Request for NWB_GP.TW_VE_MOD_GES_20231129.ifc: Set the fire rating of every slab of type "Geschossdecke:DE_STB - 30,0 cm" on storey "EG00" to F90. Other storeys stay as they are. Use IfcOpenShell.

First a look at what the model holds.

```python
import ifcopenshell
import ifcopenshell.util.element

model = ifcopenshell.open("NWB_GP.TW_VE_MOD_GES_20231129.ifc")
print(model.schema)
storey = next(s for s in model.by_type("IfcBuildingStorey") if s.Name == "EG00")
slabs = [e for e in ifcopenshell.util.element.get_decomposition(storey) if e.is_a("IfcSlab")]
seen = {}
for e in slabs:
    element_type = ifcopenshell.util.element.get_type(e)
    key = (element_type.Name if element_type != e and element_type else None, ifcopenshell.util.element.get_pset(e, "Pset_SlabCommon", "FireRating"))
    seen[key] = seen.get(key, 0) + 1
for (name, value), count in sorted(seen.items(), key=str):
    print(count, "x", name, "|", value)
```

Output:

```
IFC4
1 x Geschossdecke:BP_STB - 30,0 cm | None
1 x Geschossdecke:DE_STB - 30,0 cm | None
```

```python
import ifcopenshell
import ifcopenshell.api.pset
import ifcopenshell.util.element

model = ifcopenshell.open("NWB_GP.TW_VE_MOD_GES_20231129.ifc")

storey = next(s for s in model.by_type("IfcBuildingStorey") if s.Name == "EG00")
slabs = [e for e in ifcopenshell.util.element.get_decomposition(storey) if e.is_a("IfcSlab")]

count = 0
for e in slabs:
    element_type = ifcopenshell.util.element.get_type(e)
    if element_type in (None, e) or element_type.Name != "Geschossdecke:DE_STB - 30,0 cm":
        continue
    # add_pset returns the element's existing set when there is one.
    pset = ifcopenshell.api.pset.add_pset(model, product=e, name="Pset_SlabCommon")
    ifcopenshell.api.pset.edit_pset(model, pset=pset, properties={"FireRating": "F90"})
    count += 1

print(count, "slabs updated")

model.write("NWB_GP.TW_VE_MOD_GES_20231129-out.ifc")
```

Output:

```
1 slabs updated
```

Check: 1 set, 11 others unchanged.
